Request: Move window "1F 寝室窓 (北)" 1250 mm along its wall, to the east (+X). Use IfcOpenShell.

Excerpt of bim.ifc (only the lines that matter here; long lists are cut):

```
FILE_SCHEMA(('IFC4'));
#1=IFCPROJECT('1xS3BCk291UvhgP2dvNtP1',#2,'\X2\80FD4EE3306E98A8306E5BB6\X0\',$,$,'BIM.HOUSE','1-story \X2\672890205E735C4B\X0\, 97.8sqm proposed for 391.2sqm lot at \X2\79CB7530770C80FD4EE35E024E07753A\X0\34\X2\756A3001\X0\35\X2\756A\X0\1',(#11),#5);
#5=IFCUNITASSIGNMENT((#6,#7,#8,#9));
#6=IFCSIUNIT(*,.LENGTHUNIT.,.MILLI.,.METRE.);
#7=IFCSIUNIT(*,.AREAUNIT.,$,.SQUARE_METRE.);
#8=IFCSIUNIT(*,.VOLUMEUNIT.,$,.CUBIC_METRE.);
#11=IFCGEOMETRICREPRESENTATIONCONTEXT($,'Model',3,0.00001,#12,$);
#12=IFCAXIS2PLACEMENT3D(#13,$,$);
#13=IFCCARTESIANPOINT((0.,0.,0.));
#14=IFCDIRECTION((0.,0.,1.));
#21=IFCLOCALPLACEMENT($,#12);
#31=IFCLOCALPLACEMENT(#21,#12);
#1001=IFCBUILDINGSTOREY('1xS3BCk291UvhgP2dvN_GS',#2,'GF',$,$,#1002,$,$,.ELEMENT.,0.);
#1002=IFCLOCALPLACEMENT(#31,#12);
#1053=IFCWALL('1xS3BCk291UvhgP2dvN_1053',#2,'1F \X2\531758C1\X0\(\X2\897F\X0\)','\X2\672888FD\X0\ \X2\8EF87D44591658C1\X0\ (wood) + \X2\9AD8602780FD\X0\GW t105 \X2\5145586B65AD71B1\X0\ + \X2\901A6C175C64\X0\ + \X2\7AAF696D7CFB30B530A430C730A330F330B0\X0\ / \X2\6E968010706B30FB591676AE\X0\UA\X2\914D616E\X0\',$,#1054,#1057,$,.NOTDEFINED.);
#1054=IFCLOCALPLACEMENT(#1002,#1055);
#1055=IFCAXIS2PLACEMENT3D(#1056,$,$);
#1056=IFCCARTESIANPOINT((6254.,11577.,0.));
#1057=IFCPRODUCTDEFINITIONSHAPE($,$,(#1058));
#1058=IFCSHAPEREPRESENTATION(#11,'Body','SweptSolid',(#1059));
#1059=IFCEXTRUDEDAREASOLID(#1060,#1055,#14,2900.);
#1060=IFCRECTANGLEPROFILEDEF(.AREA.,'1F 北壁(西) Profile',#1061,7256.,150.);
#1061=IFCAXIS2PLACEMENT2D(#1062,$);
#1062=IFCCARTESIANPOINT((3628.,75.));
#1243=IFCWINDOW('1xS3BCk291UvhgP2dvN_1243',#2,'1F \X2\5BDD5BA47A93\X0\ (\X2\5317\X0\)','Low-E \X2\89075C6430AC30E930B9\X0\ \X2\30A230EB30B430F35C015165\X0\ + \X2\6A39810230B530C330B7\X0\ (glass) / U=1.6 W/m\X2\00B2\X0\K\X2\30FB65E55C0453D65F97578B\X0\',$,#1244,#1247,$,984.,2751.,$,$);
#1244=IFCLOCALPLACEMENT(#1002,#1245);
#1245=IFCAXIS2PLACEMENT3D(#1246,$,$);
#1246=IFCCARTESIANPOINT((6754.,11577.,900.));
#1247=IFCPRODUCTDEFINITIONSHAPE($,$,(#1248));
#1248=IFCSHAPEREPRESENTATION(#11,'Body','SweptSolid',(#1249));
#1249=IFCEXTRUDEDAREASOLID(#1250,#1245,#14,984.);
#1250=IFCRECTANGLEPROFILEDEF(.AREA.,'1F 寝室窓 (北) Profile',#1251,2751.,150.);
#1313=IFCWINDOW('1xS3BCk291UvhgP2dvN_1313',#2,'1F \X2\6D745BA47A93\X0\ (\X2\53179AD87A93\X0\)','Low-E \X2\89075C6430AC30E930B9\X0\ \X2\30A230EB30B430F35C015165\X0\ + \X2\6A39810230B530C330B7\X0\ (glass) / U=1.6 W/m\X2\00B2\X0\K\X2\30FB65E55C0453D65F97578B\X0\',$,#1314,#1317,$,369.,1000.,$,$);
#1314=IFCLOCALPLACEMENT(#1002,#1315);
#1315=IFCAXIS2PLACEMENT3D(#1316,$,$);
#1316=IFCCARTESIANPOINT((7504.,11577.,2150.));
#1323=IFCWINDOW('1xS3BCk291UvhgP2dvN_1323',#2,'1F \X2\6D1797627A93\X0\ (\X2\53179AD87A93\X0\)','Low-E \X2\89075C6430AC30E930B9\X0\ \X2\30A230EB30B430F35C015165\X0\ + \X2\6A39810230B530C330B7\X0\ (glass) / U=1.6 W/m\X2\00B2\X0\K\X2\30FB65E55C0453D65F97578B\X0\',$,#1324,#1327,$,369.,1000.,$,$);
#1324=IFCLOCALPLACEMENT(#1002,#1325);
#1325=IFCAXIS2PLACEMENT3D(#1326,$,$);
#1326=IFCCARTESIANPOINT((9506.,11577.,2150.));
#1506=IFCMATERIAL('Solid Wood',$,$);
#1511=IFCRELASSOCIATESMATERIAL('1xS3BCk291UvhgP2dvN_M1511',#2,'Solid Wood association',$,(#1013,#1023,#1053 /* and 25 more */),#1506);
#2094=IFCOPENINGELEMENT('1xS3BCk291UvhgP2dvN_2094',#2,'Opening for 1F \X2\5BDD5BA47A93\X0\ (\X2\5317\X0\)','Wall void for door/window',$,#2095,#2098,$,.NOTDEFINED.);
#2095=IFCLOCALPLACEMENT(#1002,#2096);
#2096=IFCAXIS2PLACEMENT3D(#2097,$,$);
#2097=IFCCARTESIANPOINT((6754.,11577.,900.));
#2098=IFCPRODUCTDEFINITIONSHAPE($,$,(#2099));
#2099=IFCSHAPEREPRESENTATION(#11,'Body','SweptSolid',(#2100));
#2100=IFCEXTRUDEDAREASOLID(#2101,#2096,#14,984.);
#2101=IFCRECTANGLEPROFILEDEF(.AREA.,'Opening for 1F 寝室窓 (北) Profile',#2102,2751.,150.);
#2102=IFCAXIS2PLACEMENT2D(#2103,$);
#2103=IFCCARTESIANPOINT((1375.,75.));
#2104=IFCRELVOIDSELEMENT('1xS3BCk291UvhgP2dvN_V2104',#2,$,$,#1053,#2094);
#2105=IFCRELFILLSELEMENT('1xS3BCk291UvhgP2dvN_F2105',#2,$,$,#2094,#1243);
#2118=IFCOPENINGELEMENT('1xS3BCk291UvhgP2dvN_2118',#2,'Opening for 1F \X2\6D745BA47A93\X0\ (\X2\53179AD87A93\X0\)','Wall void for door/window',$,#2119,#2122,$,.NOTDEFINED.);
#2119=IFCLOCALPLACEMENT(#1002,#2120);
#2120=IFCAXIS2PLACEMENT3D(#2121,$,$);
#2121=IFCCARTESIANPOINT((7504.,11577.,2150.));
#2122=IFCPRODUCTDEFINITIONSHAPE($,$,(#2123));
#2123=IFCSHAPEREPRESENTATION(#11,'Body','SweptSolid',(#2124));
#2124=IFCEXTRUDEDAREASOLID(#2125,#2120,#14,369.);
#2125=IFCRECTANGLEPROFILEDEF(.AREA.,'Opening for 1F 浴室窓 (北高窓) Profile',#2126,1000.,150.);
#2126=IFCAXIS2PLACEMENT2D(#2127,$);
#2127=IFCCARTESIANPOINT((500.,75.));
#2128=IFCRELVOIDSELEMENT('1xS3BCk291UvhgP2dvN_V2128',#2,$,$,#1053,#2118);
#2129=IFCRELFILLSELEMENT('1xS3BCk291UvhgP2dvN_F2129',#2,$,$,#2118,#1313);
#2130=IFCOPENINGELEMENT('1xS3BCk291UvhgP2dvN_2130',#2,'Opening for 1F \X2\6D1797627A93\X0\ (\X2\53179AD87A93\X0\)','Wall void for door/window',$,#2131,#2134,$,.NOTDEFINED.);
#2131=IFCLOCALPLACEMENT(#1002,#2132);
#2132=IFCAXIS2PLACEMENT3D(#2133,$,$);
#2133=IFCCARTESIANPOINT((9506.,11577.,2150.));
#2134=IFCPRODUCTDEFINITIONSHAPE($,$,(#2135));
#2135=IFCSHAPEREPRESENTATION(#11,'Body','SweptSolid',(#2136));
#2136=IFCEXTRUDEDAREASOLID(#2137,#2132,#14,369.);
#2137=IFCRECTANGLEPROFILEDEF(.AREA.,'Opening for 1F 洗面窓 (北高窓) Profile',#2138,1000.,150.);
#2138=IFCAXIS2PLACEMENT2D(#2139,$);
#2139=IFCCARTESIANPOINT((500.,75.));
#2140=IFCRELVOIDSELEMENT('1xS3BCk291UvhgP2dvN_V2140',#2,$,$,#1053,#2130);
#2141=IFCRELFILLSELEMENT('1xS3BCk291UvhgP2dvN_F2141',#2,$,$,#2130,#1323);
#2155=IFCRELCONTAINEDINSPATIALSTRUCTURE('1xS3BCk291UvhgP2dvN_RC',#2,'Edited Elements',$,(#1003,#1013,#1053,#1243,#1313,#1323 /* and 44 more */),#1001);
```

```python
import ifcopenshell
import ifcopenshell.api.geometry
import ifcopenshell.util.placement
import ifcopenshell.util.unit

model = ifcopenshell.open("bim.ifc")
unit_scale = ifcopenshell.util.unit.calculate_unit_scale(model)

window = model.by_guid("1xS3BCk291UvhgP2dvN_1243")
opening = window.FillsVoids[0].RelatingOpeningElement
wall = opening.VoidsElements[0].RelatingBuildingElement

wall_matrix = ifcopenshell.util.placement.get_local_placement(wall.ObjectPlacement)
shift = wall_matrix[:3, 0] * 1.25 / unit_scale
before = ifcopenshell.util.placement.get_local_placement(window.ObjectPlacement)[:3, 3].copy()

# The window is not placed relative to its opening, so move both.
for product in (opening, window):
    matrix = ifcopenshell.util.placement.get_local_placement(product.ObjectPlacement)
    matrix[:3, 3] += shift
    ifcopenshell.api.geometry.edit_object_placement(model, product=product, matrix=matrix, is_si=False)

after = ifcopenshell.util.placement.get_local_placement(window.ObjectPlacement)[:3, 3]
print("window moved by", (after - before).round(3) + 0.0)

model.write("bim-out.ifc")
```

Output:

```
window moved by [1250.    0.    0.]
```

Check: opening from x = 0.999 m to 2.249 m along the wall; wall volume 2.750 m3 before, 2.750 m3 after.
